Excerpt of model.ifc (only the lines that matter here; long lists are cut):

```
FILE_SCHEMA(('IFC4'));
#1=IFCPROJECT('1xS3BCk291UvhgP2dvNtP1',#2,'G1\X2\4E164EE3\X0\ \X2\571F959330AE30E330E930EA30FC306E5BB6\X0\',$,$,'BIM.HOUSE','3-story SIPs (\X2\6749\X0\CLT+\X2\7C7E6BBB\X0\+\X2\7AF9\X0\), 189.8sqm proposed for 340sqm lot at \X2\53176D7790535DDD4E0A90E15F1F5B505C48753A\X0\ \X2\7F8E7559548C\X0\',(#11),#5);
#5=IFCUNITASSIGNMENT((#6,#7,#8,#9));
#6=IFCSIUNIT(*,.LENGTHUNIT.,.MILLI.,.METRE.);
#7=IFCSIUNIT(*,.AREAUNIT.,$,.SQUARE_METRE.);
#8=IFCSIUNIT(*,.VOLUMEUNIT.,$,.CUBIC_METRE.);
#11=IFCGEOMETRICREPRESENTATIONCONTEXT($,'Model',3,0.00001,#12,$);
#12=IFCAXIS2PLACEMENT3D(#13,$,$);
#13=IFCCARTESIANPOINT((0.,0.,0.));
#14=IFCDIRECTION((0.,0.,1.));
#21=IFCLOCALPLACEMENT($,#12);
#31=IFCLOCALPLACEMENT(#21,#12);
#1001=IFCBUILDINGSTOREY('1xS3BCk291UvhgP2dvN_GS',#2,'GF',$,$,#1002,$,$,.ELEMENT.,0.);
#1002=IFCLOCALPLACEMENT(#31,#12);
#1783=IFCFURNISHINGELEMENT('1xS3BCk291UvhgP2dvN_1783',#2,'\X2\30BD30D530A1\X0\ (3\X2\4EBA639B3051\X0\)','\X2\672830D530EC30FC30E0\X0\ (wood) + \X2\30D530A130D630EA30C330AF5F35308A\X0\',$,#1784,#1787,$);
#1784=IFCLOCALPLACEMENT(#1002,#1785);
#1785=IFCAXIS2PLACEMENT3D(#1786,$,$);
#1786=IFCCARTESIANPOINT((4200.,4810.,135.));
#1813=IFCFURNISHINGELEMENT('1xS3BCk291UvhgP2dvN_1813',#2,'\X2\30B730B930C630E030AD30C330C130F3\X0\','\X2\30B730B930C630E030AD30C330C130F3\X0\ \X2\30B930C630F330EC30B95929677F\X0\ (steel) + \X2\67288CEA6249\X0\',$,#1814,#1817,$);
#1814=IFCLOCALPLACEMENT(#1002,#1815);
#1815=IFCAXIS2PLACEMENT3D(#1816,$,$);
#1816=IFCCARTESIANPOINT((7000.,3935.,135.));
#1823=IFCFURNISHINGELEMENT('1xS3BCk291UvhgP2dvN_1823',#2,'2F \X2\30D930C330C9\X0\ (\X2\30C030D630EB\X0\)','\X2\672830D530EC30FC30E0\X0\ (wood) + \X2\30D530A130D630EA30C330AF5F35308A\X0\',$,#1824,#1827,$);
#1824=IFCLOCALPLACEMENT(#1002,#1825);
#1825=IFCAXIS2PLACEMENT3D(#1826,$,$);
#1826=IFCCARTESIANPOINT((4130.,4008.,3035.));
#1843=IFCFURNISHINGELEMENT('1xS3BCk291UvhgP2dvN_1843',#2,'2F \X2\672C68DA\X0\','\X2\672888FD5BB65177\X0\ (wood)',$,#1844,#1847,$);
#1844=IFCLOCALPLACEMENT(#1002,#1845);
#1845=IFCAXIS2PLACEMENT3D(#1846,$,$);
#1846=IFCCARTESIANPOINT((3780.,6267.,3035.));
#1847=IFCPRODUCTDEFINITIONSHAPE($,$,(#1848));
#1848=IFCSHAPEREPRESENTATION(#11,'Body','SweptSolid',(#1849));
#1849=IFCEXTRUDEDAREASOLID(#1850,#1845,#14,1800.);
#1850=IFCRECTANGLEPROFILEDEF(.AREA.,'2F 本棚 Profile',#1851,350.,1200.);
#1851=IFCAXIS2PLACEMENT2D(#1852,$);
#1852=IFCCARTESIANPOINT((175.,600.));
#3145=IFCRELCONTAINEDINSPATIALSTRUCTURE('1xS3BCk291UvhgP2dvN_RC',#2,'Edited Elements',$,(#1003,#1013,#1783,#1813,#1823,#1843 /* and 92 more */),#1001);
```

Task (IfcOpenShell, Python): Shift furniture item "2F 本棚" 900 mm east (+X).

```python
import ifcopenshell
import ifcopenshell.api.geometry
import ifcopenshell.util.placement
import ifcopenshell.util.unit

model = ifcopenshell.open("model.ifc")
unit_scale = ifcopenshell.util.unit.calculate_unit_scale(model)

item = model.by_id(1843)
matrix = ifcopenshell.util.placement.get_local_placement(item.ObjectPlacement)
matrix[0, 3] += 0.9 / unit_scale
ifcopenshell.api.geometry.edit_object_placement(model, product=item, matrix=matrix, is_si=False)

print(ifcopenshell.util.placement.get_local_placement(item.ObjectPlacement).round(3) + 0.0)

model.write("model_updated.ifc")
```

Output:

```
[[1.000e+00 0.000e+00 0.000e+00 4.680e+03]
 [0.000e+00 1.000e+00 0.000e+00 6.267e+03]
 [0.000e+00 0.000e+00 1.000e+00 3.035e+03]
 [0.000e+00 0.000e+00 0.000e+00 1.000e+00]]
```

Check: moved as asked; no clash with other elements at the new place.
